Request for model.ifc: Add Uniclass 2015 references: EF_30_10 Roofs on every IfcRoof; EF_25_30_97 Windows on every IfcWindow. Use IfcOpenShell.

First a look at what the model holds.

```python
import ifcopenshell

model = ifcopenshell.open("model.ifc")
print(model.schema)
print("classifications:", [c.Name for c in model.by_type("IfcClassification")])
for ifc_class in ("IfcDoor", "IfcRoof", "IfcStair", "IfcWall", "IfcWindow"):
    print(ifc_class, len(model.by_type(ifc_class)))
```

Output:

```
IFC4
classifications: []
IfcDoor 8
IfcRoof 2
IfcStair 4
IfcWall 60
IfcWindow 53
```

```python
import ifcopenshell
import ifcopenshell.api.classification

model = ifcopenshell.open("model.ifc")

system = ifcopenshell.api.classification.add_classification(model, classification="Uniclass 2015")

codes = {
    "IfcRoof": ("EF_30_10", "Roofs"),
    "IfcWindow": ("EF_25_30_97", "Windows"),
}
for ifc_class, (code, name) in codes.items():
    products = model.by_type(ifc_class)
    ifcopenshell.api.classification.add_reference(
        model, products=products, classification=system, identification=code, name=name
    )
    print(code, len(products))

model.write("model_edited.ifc")
```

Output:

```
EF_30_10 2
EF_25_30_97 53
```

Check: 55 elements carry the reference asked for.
